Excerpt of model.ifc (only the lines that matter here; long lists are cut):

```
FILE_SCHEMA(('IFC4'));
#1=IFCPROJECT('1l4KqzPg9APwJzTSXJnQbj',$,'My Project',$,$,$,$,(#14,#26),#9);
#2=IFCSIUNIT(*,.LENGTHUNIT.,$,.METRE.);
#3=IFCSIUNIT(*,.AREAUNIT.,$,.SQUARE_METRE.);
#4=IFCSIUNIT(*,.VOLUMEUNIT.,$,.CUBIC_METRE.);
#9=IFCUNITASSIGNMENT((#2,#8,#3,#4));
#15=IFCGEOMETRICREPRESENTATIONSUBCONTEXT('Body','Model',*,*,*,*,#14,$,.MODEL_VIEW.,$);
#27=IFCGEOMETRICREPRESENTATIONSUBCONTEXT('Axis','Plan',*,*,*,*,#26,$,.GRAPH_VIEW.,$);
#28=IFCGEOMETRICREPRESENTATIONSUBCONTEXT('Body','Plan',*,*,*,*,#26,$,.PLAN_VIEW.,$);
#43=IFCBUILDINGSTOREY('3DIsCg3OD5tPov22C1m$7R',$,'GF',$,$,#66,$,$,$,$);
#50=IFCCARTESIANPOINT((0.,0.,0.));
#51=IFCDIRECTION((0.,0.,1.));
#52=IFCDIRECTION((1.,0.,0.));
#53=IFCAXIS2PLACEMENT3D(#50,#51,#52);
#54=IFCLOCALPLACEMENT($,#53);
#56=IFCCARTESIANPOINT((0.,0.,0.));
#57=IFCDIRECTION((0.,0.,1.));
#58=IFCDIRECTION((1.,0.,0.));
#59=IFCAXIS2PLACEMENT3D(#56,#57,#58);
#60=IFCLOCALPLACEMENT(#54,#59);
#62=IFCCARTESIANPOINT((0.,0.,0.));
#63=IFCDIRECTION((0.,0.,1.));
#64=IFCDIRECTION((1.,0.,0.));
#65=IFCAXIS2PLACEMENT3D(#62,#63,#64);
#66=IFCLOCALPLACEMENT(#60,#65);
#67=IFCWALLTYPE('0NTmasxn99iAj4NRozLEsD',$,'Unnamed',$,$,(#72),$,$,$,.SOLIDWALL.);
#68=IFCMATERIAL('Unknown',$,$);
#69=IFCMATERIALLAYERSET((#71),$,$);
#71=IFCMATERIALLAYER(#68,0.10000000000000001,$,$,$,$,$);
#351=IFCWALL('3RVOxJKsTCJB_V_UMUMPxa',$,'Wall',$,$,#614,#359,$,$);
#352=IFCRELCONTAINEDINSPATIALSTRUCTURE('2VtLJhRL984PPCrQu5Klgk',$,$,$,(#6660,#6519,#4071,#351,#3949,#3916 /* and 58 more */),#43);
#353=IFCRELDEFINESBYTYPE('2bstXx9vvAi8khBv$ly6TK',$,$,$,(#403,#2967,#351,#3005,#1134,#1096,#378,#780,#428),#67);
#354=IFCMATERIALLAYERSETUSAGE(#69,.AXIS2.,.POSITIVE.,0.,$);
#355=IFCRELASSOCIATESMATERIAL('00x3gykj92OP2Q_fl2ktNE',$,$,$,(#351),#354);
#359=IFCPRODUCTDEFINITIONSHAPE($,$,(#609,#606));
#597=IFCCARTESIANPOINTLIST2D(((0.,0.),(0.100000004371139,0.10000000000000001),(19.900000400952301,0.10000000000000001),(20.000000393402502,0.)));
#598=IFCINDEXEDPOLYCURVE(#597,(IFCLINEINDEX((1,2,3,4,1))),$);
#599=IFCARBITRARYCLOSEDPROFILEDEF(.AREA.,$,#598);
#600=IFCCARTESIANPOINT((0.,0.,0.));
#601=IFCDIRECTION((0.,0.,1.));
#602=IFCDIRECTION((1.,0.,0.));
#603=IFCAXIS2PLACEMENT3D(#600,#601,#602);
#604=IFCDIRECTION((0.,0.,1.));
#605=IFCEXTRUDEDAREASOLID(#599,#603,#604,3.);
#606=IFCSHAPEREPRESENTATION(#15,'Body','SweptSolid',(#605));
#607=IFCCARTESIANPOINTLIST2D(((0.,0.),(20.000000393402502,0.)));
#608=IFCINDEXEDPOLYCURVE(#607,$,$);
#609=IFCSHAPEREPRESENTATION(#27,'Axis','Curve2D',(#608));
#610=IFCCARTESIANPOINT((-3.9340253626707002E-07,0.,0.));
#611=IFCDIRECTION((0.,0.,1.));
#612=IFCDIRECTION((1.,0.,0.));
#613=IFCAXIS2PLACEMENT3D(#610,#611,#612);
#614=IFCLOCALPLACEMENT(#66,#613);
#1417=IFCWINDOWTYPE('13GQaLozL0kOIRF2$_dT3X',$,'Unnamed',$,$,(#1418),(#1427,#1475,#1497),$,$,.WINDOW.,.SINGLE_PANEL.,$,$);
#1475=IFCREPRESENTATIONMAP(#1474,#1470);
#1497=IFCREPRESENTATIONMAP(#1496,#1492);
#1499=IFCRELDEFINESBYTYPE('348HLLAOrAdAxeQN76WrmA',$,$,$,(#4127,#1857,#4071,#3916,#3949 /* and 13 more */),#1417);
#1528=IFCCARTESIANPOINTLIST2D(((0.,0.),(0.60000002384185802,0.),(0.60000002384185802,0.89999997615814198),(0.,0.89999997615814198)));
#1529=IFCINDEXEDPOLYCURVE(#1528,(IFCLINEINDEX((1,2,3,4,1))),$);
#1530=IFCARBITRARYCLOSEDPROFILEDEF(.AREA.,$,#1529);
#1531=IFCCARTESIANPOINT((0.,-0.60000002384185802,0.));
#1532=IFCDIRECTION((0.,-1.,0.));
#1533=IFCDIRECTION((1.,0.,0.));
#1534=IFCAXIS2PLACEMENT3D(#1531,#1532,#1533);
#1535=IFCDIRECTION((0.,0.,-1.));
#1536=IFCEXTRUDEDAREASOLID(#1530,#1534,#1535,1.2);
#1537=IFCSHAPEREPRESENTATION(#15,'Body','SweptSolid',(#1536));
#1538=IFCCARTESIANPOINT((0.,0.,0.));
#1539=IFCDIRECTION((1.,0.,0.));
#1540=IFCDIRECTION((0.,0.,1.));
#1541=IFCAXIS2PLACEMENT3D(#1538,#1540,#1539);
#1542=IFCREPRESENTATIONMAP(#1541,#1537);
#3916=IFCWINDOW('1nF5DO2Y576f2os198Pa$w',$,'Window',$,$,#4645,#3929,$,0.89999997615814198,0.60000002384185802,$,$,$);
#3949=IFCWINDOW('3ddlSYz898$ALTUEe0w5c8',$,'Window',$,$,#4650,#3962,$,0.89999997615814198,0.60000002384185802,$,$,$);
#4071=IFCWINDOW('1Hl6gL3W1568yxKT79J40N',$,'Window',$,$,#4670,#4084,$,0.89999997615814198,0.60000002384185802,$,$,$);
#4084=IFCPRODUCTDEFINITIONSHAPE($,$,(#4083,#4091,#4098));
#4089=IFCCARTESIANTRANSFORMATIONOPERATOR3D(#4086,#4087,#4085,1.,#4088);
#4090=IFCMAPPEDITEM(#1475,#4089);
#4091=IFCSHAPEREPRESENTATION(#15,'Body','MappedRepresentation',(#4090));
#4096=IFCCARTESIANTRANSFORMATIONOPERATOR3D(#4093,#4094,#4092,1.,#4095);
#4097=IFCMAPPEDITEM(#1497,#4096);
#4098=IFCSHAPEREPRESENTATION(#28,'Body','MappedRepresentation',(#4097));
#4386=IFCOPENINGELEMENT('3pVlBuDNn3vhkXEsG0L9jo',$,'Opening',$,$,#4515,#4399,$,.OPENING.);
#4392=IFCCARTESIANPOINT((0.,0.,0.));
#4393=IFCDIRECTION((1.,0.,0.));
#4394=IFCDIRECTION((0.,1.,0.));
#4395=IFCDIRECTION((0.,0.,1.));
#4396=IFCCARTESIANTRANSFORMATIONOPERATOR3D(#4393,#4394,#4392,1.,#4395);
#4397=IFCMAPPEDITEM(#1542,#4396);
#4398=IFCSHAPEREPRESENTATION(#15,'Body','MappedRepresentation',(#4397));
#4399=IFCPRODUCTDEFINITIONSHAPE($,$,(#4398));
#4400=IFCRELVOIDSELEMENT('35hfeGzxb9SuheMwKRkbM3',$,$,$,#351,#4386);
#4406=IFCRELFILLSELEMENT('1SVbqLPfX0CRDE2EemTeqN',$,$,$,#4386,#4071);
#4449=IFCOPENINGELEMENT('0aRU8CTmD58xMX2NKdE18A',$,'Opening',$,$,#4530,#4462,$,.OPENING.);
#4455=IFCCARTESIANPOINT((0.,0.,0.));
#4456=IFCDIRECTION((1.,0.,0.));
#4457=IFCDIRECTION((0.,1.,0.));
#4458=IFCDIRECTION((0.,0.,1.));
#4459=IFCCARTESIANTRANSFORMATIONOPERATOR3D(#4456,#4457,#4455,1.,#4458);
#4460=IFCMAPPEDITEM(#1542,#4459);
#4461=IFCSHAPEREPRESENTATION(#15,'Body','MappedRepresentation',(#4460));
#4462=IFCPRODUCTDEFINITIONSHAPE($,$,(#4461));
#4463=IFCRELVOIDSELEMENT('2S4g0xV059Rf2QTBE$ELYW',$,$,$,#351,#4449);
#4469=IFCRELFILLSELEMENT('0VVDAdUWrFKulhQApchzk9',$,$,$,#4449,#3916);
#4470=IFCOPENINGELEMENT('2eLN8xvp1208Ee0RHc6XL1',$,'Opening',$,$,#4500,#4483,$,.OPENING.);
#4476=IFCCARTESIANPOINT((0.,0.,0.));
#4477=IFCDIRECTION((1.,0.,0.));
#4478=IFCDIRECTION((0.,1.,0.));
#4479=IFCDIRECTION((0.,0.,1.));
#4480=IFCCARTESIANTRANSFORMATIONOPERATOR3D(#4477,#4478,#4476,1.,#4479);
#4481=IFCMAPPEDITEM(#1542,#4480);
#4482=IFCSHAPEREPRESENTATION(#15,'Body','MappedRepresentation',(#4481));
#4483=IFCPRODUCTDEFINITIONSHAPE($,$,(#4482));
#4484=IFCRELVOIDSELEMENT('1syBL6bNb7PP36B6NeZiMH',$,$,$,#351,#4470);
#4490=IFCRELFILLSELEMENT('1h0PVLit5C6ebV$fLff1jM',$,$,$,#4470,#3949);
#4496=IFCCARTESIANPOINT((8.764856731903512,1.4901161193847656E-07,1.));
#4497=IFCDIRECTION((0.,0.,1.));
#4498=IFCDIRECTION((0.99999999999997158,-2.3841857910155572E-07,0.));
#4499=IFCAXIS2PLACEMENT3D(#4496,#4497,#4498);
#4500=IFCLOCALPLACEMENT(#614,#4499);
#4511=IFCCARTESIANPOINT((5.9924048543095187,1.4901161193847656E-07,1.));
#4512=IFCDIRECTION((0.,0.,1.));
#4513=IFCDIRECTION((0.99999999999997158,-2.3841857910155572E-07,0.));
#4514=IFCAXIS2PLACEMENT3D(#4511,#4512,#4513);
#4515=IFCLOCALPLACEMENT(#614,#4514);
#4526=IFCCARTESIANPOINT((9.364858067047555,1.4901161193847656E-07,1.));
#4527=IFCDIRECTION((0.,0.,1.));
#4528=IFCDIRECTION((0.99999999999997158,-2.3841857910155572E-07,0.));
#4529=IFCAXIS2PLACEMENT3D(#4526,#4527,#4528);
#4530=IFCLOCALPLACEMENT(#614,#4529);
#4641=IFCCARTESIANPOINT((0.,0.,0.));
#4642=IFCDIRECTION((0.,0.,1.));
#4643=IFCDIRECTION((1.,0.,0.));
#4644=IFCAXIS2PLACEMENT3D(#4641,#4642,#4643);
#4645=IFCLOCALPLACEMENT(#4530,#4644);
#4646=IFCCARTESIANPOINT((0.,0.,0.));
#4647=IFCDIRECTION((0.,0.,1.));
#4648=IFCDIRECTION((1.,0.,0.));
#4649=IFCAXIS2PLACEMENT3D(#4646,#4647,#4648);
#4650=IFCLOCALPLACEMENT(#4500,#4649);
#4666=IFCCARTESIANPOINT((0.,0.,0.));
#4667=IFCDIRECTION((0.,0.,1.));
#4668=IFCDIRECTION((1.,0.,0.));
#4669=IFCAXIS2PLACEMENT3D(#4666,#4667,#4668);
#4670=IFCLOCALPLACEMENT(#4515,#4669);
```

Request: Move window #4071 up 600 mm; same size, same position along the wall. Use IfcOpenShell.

```python
import numpy as np
import ifcopenshell
import ifcopenshell.api.geometry
import ifcopenshell.util.placement
import ifcopenshell.util.unit

model = ifcopenshell.open("model.ifc")
unit_scale = ifcopenshell.util.unit.calculate_unit_scale(model)

window = model.by_id(4071)
opening = window.FillsVoids[0].RelatingOpeningElement
dz = 0.6

shift = np.array([0.0, 0.0, dz])
# The window is placed relative to its opening, so it follows when the opening moves.
matrix = ifcopenshell.util.placement.get_local_placement(opening.ObjectPlacement)
matrix[:3, 3] += shift
ifcopenshell.api.geometry.edit_object_placement(
    model, product=opening, matrix=matrix, is_si=False, should_transform_children=True
)

print(f"moved by {dz * unit_scale:+.3f} m")

model.write("model-out.ifc")
```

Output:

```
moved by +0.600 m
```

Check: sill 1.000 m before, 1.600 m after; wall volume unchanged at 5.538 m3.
